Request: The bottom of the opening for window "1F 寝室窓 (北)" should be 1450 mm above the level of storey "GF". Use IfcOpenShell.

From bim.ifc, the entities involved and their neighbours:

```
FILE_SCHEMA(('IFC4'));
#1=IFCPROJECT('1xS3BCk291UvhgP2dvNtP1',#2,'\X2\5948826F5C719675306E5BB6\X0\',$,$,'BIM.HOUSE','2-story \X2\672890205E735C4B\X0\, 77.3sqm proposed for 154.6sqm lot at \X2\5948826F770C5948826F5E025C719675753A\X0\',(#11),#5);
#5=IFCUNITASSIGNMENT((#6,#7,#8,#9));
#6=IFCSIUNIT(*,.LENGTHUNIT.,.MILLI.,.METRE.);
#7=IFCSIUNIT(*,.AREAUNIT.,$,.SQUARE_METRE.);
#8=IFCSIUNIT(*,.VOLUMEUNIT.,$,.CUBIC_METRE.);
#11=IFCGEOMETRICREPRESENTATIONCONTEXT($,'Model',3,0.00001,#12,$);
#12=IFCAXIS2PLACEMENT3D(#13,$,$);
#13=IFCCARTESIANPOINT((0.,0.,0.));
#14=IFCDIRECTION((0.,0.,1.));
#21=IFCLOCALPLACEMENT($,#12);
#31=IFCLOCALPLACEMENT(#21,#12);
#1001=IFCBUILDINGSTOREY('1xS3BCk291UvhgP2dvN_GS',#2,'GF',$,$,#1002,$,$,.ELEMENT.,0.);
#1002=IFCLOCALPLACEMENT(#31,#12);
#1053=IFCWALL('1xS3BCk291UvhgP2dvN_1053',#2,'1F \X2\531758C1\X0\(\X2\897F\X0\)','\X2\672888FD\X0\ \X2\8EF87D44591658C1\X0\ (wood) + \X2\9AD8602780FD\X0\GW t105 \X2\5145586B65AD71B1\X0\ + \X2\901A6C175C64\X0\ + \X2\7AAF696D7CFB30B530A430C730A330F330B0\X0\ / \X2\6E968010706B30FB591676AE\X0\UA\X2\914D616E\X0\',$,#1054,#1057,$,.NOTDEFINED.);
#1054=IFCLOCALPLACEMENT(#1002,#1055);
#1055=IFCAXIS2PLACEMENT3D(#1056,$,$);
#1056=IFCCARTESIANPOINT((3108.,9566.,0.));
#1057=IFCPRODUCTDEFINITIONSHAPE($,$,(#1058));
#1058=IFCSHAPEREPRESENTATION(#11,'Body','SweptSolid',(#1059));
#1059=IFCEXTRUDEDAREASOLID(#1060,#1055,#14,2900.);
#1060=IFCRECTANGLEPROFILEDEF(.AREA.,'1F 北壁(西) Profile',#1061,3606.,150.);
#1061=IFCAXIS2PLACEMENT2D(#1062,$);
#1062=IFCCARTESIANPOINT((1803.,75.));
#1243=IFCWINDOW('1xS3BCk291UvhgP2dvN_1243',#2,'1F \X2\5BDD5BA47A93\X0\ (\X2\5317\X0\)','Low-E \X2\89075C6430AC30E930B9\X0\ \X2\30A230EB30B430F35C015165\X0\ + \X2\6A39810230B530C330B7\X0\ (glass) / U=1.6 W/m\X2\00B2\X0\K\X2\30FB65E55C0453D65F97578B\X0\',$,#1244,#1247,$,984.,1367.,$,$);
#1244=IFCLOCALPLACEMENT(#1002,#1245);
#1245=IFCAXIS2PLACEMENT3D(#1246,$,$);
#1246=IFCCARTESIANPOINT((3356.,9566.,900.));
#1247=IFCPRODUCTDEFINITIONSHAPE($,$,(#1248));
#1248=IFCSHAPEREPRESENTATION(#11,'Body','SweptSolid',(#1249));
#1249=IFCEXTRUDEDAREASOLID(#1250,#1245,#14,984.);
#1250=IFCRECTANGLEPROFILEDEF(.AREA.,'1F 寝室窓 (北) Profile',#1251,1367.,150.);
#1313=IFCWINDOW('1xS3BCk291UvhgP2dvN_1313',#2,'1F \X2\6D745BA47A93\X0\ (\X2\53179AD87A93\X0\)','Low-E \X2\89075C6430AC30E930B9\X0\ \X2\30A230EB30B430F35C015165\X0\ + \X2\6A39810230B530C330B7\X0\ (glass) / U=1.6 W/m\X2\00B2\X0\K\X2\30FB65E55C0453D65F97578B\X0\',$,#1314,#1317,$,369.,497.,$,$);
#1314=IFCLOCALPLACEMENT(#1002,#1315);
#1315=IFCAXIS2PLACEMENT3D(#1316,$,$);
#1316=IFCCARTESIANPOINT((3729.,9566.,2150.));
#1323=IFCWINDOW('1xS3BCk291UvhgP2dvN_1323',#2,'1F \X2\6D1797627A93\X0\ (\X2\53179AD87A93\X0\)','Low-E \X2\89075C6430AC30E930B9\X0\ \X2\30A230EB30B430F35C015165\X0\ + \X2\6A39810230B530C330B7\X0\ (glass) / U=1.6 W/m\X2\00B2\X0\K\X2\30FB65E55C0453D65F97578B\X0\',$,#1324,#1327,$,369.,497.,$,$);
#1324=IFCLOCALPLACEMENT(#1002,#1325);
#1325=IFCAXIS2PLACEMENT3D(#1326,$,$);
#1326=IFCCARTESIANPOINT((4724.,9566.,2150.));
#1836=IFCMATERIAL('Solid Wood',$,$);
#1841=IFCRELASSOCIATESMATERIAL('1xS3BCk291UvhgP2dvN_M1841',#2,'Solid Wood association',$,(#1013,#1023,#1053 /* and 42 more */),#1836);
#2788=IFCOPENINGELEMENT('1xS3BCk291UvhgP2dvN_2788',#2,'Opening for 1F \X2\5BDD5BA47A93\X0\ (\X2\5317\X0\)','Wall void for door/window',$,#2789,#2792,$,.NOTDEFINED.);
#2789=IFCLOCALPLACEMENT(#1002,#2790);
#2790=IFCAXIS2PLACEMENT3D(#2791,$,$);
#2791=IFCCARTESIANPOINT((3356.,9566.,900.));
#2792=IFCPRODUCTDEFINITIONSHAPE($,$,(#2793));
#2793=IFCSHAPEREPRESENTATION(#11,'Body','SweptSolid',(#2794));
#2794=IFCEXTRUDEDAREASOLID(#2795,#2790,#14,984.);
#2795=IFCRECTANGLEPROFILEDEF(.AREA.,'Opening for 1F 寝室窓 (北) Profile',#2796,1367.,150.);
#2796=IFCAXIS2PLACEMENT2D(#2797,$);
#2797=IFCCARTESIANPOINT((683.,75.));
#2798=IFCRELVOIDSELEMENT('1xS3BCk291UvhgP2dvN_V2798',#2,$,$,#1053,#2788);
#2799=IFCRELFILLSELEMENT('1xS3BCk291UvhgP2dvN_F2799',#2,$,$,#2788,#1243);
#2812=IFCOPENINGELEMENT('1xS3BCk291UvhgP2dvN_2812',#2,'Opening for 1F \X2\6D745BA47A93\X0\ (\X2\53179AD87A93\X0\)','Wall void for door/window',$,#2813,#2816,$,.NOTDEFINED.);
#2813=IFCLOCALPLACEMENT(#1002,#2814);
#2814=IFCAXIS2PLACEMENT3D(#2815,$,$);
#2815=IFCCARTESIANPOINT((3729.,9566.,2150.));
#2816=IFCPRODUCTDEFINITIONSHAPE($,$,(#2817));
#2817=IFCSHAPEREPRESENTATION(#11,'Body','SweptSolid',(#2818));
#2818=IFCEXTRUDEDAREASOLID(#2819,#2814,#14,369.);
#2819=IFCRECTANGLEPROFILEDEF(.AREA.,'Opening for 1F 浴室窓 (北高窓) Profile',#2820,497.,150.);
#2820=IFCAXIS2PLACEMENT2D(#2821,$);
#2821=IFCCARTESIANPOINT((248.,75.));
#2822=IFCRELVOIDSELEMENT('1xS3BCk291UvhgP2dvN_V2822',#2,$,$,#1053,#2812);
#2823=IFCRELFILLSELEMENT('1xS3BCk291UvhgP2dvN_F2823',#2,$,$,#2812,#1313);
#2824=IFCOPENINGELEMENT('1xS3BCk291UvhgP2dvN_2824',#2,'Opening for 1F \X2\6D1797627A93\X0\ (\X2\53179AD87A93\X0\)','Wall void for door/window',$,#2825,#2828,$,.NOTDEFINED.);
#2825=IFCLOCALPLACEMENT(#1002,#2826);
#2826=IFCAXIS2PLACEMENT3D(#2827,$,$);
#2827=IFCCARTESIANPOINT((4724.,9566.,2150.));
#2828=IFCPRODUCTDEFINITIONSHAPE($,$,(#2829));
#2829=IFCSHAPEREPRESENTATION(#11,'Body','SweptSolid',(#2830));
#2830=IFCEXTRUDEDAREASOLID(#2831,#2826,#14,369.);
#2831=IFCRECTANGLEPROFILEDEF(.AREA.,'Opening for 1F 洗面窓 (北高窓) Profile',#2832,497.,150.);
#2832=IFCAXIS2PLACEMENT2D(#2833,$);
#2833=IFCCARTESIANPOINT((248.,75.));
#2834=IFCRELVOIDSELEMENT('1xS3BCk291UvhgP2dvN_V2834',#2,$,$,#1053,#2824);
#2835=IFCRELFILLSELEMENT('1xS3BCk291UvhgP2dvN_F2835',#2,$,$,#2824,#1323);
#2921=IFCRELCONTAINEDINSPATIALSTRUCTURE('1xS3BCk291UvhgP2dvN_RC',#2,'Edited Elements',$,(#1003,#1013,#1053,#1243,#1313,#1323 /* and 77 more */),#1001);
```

```python
import numpy as np
import ifcopenshell
import ifcopenshell.api.geometry
import ifcopenshell.geom
import ifcopenshell.util.element
import ifcopenshell.util.placement
import ifcopenshell.util.shape
import ifcopenshell.util.unit

model = ifcopenshell.open("bim.ifc")
unit_scale = ifcopenshell.util.unit.calculate_unit_scale(model)

window = model.by_guid("1xS3BCk291UvhgP2dvN_1243")
opening = window.FillsVoids[0].RelatingOpeningElement
storey = ifcopenshell.util.element.get_container(window, ifc_class="IfcBuildingStorey")
level = ifcopenshell.util.placement.get_local_placement(storey.ObjectPlacement)[2, 3]

# The opening's origin need not be at the sill, so measure its lowest point.
shape = ifcopenshell.geom.create_shape(ifcopenshell.geom.settings(), opening)
bottom = ifcopenshell.util.shape.get_shape_bottom_elevation(shape, shape.geometry) / unit_scale
dz = level + 1.45 / unit_scale - bottom

shift = np.array([0.0, 0.0, dz])
# The window is not placed relative to its opening, so move both.
for product in (opening, window):
    matrix = ifcopenshell.util.placement.get_local_placement(product.ObjectPlacement)
    matrix[:3, 3] += shift
    ifcopenshell.api.geometry.edit_object_placement(model, product=product, matrix=matrix, is_si=False)

print(f"moved by {dz * unit_scale:+.3f} m")

model.write("bim-out.ifc")
```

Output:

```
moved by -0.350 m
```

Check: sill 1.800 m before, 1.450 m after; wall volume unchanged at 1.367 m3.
